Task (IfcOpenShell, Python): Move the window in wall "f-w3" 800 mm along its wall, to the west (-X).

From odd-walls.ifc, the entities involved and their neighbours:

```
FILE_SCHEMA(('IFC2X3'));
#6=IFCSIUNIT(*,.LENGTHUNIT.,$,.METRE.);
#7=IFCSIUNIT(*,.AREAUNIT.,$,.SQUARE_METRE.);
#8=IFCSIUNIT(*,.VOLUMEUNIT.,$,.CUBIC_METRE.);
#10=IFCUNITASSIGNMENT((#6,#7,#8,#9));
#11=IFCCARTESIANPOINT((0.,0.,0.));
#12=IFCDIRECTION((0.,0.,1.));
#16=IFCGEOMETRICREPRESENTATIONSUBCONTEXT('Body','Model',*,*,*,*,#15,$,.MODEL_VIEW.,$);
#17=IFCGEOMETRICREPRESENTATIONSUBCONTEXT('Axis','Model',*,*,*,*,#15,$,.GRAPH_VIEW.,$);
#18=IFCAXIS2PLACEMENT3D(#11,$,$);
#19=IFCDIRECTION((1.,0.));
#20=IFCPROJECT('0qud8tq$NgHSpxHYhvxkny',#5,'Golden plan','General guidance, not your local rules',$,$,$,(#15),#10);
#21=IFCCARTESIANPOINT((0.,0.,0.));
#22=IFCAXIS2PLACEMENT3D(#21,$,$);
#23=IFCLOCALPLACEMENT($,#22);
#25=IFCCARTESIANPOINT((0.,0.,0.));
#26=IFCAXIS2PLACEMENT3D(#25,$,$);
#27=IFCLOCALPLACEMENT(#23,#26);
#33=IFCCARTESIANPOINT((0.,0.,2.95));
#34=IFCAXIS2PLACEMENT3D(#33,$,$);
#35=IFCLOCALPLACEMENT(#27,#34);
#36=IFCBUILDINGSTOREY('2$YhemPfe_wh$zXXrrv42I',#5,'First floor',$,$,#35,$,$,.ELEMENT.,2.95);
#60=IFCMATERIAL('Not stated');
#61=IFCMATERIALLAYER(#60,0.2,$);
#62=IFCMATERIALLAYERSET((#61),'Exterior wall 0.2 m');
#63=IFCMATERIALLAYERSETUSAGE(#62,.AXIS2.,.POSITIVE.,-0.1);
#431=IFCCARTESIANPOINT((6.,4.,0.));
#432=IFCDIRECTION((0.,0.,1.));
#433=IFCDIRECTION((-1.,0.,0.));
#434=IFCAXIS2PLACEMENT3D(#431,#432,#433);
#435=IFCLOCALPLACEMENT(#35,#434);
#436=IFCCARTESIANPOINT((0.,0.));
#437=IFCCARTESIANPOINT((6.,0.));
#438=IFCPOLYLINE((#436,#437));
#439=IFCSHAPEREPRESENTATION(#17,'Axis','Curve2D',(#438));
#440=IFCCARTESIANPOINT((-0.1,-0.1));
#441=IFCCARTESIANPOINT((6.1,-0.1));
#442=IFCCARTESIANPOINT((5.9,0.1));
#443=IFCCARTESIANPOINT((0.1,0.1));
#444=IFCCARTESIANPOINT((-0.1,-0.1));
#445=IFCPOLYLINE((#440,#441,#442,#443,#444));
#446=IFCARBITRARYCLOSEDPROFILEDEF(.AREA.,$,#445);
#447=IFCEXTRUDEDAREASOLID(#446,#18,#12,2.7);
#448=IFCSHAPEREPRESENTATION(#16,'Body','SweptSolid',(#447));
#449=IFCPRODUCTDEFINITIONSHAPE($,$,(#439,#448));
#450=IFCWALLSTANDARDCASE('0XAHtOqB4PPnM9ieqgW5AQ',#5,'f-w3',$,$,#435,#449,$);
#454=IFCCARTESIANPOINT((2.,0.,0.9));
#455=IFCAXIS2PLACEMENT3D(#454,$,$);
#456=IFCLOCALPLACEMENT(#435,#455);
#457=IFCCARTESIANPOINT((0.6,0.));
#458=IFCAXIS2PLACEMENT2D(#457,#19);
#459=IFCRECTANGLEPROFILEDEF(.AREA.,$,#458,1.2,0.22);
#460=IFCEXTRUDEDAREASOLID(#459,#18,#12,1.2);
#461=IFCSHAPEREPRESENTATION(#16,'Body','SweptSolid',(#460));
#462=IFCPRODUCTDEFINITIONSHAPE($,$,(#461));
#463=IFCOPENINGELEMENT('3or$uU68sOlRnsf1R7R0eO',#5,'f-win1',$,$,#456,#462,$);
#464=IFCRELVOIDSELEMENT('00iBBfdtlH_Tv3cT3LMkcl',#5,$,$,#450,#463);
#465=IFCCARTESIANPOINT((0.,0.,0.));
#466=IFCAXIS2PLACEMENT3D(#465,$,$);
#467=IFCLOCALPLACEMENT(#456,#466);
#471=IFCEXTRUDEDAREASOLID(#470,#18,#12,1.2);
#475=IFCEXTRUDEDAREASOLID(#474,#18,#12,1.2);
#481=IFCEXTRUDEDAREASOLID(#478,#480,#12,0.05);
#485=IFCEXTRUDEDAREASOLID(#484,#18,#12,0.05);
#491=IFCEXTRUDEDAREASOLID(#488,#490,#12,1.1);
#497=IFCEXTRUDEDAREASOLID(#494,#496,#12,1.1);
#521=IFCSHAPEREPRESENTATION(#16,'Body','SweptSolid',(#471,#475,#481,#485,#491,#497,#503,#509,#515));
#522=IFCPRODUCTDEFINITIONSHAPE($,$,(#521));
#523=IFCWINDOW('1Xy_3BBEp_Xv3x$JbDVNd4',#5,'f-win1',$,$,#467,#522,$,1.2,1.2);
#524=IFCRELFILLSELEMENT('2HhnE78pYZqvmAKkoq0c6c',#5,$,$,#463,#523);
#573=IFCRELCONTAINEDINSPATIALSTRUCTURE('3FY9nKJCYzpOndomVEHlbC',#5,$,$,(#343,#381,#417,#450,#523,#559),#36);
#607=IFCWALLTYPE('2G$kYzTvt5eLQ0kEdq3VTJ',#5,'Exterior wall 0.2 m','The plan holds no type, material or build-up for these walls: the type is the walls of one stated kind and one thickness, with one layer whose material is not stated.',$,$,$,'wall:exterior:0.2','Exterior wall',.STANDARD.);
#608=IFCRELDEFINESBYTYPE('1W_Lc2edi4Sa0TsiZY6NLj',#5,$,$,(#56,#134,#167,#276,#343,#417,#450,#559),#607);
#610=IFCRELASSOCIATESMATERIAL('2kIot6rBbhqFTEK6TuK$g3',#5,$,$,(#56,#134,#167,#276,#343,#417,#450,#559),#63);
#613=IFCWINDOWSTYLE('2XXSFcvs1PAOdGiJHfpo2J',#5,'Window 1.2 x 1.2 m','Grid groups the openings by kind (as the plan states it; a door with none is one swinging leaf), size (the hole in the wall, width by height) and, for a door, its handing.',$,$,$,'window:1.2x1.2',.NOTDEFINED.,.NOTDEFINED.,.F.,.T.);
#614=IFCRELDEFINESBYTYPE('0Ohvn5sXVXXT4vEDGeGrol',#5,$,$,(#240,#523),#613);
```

```python
import ifcopenshell
import ifcopenshell.api.geometry
import ifcopenshell.util.placement
import ifcopenshell.util.unit

model = ifcopenshell.open("odd-walls.ifc")
unit_scale = ifcopenshell.util.unit.calculate_unit_scale(model)

window = model.by_guid("1Xy_3BBEp_Xv3x$JbDVNd4")
opening = window.FillsVoids[0].RelatingOpeningElement
wall = opening.VoidsElements[0].RelatingBuildingElement

wall_matrix = ifcopenshell.util.placement.get_local_placement(wall.ObjectPlacement)
shift = wall_matrix[:3, 0] * 0.8 / unit_scale
before = ifcopenshell.util.placement.get_local_placement(window.ObjectPlacement)[:3, 3].copy()

# The window is placed relative to its opening, so it follows when the opening moves.
matrix = ifcopenshell.util.placement.get_local_placement(opening.ObjectPlacement)
matrix[:3, 3] += shift
ifcopenshell.api.geometry.edit_object_placement(
    model, product=opening, matrix=matrix, is_si=False, should_transform_children=True
)

after = ifcopenshell.util.placement.get_local_placement(window.ObjectPlacement)[:3, 3]
print("window moved by", (after - before).round(3) + 0.0)

model.write("odd-walls_updated.ifc")
```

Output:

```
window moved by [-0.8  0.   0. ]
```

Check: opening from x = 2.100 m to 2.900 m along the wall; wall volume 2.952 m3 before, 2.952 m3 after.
